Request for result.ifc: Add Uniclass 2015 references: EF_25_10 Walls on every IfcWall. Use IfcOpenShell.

First a look at what the model holds.

```python
import ifcopenshell

model = ifcopenshell.open("result.ifc")
print(model.schema)
print("classifications:", [c.Name for c in model.by_type("IfcClassification")])
for ifc_class in ("IfcDoor", "IfcRoof", "IfcStair", "IfcWall", "IfcWindow"):
    print(ifc_class, len(model.by_type(ifc_class)))
```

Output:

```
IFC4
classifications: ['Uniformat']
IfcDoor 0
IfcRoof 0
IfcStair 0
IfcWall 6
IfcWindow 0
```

```python
import ifcopenshell
import ifcopenshell.api.classification

model = ifcopenshell.open("result.ifc")

system = ifcopenshell.api.classification.add_classification(model, classification="Uniclass 2015")

codes = {
    "IfcWall": ("EF_25_10", "Walls"),
}
for ifc_class, (code, name) in codes.items():
    products = model.by_type(ifc_class)
    ifcopenshell.api.classification.add_reference(
        model, products=products, classification=system, identification=code, name=name
    )
    print(code, len(products))

model.write("result_edited.ifc")
```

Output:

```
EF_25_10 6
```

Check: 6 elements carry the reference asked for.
